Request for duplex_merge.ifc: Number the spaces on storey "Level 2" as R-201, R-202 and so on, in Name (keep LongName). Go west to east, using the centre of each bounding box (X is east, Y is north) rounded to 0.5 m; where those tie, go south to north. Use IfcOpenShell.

First a look at what the model holds.

```python
import ifcopenshell
import ifcopenshell.util.element
import ifcopenshell.util.placement

model = ifcopenshell.open("duplex_merge.ifc")
print(model.schema)
storey = next(s for s in model.by_type("IfcBuildingStorey") if s.Name == "Level 2")
spaces = [e for e in ifcopenshell.util.element.get_decomposition(storey) if e.is_a("IfcSpace")]
for e in sorted(spaces, key=lambda e: e.id()):
    origin = ifcopenshell.util.placement.get_local_placement(e.ObjectPlacement)[:3, 3]
    print(e.id(), e.Name, e.LongName, origin.round(2) + 0.0, sep=" | ")
```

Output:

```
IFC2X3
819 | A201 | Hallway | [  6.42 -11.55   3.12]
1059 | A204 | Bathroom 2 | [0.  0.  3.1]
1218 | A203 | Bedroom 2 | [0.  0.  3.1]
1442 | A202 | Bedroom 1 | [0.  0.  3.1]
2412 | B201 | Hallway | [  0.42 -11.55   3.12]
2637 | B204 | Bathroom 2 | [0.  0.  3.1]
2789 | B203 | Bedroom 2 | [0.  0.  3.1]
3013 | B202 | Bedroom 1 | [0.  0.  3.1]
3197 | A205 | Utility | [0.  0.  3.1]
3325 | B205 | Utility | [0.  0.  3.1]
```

```python
import ifcopenshell
import ifcopenshell.geom
import ifcopenshell.util.element
import ifcopenshell.util.shape

model = ifcopenshell.open("duplex_merge.ifc")
settings = ifcopenshell.geom.settings()
settings.set("use-world-coords", True)


def centre(element):
    shape = ifcopenshell.geom.create_shape(settings, element)
    return ifcopenshell.util.shape.get_bbox_centroid(shape.geometry)


storey = next(s for s in model.by_type("IfcBuildingStorey") if s.Name == "Level 2")
spaces = [e for e in ifcopenshell.util.element.get_decomposition(storey) if e.is_a("IfcSpace")]

# Insertion points can sit at a corner or the storey origin, so sort by the geometry (in metres).
centres = {e: centre(e) for e in spaces}
spaces.sort(key=lambda e: (round(centres[e][0] / 0.5), centres[e][1]))

for i, e in enumerate(spaces, start=1):
    number = f"R-2{i:02d}"
    e.Name = number
    print(e.id(), number)

model.write("duplex_merge-out.ifc")
```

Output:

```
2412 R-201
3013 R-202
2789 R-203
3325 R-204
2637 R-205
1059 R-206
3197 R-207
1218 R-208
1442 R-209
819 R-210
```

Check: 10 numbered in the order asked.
